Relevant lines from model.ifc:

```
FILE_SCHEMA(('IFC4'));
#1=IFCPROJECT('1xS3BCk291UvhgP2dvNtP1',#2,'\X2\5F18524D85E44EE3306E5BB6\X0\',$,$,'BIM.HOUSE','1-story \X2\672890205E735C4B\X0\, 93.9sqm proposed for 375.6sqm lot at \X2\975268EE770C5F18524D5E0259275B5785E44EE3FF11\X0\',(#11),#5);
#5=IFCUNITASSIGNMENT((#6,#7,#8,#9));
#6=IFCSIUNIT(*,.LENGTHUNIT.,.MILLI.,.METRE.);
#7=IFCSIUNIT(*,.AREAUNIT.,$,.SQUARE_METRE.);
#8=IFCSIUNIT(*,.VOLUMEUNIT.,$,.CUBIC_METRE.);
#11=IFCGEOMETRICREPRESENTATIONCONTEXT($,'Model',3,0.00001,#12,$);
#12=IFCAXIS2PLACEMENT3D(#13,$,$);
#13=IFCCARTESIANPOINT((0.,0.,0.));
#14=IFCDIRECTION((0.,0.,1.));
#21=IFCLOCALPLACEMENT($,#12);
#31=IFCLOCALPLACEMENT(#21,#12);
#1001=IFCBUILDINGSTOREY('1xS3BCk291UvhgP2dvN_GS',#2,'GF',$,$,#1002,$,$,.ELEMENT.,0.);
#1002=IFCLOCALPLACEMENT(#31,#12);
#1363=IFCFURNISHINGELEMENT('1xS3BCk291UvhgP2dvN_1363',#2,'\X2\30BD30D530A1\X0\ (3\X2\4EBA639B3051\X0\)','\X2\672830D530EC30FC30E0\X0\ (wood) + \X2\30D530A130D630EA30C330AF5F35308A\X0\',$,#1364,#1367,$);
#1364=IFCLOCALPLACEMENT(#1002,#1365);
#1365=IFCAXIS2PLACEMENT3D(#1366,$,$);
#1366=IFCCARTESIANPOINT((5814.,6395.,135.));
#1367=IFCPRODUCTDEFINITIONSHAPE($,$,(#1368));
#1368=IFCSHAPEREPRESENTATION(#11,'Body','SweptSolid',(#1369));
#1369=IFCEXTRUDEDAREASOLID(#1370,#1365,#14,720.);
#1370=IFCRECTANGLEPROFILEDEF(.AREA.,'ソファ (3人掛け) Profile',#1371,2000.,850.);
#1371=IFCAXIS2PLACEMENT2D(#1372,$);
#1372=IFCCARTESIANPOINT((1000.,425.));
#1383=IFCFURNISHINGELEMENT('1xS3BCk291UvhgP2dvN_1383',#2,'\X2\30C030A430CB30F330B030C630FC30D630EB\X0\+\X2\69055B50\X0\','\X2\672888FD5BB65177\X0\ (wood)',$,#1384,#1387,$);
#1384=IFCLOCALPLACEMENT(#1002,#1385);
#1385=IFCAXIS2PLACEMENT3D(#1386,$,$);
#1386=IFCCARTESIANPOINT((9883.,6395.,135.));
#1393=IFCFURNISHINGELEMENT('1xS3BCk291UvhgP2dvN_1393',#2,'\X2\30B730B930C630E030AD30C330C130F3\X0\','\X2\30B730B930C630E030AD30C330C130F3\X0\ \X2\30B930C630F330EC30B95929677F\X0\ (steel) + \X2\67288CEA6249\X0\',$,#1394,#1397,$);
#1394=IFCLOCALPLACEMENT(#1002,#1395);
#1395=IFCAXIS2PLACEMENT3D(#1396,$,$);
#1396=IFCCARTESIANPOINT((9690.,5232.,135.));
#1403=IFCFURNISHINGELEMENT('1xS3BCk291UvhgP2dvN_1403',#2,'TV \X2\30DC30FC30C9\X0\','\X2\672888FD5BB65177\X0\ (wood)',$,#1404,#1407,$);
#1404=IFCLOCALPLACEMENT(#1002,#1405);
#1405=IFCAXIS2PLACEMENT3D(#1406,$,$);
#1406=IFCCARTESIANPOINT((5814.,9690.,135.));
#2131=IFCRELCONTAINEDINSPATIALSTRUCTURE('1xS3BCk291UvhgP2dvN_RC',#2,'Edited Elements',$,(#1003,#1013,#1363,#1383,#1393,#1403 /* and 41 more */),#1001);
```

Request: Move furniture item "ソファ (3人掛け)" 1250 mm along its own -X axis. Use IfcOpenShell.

```python
import ifcopenshell
import ifcopenshell.api.geometry
import ifcopenshell.util.placement

model = ifcopenshell.open("model.ifc")

item = model.by_guid("1xS3BCk291UvhgP2dvN_1363")
matrix = ifcopenshell.util.placement.get_local_placement(item.ObjectPlacement)
matrix[:3, 3] -= matrix[:3, 0] * 1250.0
ifcopenshell.api.geometry.edit_object_placement(model, product=item, matrix=matrix, is_si=False)

print(ifcopenshell.util.placement.get_local_placement(item.ObjectPlacement).round(3) + 0.0)

model.write("model_v2.ifc")
```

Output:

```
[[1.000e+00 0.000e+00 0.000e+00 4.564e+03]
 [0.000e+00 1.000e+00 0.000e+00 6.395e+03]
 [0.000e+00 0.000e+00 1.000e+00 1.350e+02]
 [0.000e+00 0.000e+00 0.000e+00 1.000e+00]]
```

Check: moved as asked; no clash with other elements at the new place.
